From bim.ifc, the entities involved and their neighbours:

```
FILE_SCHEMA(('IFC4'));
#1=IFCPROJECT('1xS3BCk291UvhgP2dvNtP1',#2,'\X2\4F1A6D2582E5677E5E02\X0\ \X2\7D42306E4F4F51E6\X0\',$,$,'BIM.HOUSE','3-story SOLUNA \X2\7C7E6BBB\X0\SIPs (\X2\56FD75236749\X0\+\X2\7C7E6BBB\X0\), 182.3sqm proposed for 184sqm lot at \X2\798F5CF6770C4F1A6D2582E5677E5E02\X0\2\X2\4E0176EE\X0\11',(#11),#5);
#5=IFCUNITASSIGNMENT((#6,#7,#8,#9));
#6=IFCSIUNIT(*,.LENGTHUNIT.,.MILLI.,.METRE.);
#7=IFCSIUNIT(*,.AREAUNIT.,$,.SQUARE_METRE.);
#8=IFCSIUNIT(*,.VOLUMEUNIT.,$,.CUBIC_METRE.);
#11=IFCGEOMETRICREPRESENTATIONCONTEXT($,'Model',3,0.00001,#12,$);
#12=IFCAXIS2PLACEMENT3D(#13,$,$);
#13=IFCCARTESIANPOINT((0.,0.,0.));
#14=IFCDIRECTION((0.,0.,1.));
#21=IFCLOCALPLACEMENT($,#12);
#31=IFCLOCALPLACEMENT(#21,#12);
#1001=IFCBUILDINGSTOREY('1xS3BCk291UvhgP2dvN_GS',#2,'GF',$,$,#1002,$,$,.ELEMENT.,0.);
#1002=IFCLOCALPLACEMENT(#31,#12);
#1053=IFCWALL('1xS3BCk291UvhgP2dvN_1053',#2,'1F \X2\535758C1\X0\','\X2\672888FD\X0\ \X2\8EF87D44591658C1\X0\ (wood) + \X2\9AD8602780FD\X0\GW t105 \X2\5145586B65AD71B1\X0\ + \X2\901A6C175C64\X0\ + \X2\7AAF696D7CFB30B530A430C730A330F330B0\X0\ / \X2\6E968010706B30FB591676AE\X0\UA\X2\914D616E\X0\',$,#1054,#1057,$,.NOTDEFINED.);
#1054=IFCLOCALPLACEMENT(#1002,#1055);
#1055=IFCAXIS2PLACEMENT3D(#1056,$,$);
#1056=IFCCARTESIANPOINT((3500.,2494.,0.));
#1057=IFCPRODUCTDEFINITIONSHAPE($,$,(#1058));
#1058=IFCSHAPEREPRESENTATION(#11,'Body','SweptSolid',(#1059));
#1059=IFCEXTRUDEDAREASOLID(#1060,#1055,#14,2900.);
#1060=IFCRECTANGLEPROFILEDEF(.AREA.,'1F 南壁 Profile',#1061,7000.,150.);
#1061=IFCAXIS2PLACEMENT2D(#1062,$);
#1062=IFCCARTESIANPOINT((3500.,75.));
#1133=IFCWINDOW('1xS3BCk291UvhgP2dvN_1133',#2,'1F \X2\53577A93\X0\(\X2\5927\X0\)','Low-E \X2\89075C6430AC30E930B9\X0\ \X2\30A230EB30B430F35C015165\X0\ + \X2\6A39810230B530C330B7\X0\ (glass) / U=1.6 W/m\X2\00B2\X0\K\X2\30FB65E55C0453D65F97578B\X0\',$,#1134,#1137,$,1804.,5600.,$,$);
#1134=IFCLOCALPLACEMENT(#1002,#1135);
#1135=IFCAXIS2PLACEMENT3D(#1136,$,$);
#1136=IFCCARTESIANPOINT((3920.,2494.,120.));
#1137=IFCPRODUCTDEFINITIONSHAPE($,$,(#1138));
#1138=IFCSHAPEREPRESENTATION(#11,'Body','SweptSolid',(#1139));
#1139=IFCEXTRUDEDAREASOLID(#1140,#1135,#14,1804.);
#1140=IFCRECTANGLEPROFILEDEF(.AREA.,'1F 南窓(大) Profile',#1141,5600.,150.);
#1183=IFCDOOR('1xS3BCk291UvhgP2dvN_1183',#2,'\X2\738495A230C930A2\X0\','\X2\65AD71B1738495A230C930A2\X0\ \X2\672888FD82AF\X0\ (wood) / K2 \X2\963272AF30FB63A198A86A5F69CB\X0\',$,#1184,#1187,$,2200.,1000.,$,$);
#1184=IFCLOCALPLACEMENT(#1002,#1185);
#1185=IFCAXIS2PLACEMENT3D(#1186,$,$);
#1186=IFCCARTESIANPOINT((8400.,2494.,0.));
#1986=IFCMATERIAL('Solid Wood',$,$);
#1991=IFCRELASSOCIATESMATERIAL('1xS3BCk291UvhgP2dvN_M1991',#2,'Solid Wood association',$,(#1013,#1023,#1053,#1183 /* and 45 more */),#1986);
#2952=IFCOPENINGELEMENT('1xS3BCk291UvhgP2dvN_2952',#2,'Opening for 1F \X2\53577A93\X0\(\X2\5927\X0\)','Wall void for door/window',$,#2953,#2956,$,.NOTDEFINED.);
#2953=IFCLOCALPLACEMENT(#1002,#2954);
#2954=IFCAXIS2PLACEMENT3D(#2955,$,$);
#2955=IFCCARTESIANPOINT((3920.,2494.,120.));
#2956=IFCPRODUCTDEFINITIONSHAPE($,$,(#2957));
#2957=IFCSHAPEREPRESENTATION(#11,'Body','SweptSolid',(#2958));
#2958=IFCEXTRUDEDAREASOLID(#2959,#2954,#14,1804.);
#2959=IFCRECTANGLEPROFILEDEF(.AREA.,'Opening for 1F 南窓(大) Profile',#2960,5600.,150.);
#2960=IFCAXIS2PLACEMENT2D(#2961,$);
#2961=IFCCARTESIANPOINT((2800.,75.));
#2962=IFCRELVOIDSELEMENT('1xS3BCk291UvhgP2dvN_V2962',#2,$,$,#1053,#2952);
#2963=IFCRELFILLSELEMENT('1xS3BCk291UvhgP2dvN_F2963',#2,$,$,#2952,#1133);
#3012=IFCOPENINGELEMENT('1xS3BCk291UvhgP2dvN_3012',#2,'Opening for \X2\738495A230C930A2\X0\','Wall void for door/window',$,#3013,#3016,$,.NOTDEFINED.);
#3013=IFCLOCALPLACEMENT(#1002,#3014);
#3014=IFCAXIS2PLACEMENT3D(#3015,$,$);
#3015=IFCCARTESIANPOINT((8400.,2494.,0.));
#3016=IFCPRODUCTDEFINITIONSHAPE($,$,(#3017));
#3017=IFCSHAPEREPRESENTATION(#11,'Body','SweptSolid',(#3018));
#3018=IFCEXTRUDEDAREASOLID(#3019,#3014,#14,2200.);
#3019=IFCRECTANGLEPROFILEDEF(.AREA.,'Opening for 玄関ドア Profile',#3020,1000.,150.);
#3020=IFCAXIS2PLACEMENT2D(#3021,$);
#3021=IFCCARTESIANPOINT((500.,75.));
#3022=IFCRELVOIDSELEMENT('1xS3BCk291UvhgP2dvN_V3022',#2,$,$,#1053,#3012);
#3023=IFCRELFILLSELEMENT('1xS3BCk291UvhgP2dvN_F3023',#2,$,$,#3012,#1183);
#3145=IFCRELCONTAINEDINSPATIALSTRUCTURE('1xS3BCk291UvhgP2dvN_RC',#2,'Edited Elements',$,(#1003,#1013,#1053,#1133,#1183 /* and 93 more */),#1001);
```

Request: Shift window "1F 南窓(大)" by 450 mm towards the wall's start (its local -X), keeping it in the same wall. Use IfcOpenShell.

```python
import ifcopenshell
import ifcopenshell.api.geometry
import ifcopenshell.util.placement
import ifcopenshell.util.unit

model = ifcopenshell.open("bim.ifc")
unit_scale = ifcopenshell.util.unit.calculate_unit_scale(model)

window = model.by_guid("1xS3BCk291UvhgP2dvN_1133")
opening = window.FillsVoids[0].RelatingOpeningElement
wall = opening.VoidsElements[0].RelatingBuildingElement

wall_matrix = ifcopenshell.util.placement.get_local_placement(wall.ObjectPlacement)
shift = wall_matrix[:3, 0] * -0.45 / unit_scale
before = ifcopenshell.util.placement.get_local_placement(window.ObjectPlacement)[:3, 3].copy()

# The window is not placed relative to its opening, so move both.
for product in (opening, window):
    matrix = ifcopenshell.util.placement.get_local_placement(product.ObjectPlacement)
    matrix[:3, 3] += shift
    ifcopenshell.api.geometry.edit_object_placement(model, product=product, matrix=matrix, is_si=False)

after = ifcopenshell.util.placement.get_local_placement(window.ObjectPlacement)[:3, 3]
print("window moved by", (after - before).round(3) + 0.0)

model.write("bim-out.ifc")
```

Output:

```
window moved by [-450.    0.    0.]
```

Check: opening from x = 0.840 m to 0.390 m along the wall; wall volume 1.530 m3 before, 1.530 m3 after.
